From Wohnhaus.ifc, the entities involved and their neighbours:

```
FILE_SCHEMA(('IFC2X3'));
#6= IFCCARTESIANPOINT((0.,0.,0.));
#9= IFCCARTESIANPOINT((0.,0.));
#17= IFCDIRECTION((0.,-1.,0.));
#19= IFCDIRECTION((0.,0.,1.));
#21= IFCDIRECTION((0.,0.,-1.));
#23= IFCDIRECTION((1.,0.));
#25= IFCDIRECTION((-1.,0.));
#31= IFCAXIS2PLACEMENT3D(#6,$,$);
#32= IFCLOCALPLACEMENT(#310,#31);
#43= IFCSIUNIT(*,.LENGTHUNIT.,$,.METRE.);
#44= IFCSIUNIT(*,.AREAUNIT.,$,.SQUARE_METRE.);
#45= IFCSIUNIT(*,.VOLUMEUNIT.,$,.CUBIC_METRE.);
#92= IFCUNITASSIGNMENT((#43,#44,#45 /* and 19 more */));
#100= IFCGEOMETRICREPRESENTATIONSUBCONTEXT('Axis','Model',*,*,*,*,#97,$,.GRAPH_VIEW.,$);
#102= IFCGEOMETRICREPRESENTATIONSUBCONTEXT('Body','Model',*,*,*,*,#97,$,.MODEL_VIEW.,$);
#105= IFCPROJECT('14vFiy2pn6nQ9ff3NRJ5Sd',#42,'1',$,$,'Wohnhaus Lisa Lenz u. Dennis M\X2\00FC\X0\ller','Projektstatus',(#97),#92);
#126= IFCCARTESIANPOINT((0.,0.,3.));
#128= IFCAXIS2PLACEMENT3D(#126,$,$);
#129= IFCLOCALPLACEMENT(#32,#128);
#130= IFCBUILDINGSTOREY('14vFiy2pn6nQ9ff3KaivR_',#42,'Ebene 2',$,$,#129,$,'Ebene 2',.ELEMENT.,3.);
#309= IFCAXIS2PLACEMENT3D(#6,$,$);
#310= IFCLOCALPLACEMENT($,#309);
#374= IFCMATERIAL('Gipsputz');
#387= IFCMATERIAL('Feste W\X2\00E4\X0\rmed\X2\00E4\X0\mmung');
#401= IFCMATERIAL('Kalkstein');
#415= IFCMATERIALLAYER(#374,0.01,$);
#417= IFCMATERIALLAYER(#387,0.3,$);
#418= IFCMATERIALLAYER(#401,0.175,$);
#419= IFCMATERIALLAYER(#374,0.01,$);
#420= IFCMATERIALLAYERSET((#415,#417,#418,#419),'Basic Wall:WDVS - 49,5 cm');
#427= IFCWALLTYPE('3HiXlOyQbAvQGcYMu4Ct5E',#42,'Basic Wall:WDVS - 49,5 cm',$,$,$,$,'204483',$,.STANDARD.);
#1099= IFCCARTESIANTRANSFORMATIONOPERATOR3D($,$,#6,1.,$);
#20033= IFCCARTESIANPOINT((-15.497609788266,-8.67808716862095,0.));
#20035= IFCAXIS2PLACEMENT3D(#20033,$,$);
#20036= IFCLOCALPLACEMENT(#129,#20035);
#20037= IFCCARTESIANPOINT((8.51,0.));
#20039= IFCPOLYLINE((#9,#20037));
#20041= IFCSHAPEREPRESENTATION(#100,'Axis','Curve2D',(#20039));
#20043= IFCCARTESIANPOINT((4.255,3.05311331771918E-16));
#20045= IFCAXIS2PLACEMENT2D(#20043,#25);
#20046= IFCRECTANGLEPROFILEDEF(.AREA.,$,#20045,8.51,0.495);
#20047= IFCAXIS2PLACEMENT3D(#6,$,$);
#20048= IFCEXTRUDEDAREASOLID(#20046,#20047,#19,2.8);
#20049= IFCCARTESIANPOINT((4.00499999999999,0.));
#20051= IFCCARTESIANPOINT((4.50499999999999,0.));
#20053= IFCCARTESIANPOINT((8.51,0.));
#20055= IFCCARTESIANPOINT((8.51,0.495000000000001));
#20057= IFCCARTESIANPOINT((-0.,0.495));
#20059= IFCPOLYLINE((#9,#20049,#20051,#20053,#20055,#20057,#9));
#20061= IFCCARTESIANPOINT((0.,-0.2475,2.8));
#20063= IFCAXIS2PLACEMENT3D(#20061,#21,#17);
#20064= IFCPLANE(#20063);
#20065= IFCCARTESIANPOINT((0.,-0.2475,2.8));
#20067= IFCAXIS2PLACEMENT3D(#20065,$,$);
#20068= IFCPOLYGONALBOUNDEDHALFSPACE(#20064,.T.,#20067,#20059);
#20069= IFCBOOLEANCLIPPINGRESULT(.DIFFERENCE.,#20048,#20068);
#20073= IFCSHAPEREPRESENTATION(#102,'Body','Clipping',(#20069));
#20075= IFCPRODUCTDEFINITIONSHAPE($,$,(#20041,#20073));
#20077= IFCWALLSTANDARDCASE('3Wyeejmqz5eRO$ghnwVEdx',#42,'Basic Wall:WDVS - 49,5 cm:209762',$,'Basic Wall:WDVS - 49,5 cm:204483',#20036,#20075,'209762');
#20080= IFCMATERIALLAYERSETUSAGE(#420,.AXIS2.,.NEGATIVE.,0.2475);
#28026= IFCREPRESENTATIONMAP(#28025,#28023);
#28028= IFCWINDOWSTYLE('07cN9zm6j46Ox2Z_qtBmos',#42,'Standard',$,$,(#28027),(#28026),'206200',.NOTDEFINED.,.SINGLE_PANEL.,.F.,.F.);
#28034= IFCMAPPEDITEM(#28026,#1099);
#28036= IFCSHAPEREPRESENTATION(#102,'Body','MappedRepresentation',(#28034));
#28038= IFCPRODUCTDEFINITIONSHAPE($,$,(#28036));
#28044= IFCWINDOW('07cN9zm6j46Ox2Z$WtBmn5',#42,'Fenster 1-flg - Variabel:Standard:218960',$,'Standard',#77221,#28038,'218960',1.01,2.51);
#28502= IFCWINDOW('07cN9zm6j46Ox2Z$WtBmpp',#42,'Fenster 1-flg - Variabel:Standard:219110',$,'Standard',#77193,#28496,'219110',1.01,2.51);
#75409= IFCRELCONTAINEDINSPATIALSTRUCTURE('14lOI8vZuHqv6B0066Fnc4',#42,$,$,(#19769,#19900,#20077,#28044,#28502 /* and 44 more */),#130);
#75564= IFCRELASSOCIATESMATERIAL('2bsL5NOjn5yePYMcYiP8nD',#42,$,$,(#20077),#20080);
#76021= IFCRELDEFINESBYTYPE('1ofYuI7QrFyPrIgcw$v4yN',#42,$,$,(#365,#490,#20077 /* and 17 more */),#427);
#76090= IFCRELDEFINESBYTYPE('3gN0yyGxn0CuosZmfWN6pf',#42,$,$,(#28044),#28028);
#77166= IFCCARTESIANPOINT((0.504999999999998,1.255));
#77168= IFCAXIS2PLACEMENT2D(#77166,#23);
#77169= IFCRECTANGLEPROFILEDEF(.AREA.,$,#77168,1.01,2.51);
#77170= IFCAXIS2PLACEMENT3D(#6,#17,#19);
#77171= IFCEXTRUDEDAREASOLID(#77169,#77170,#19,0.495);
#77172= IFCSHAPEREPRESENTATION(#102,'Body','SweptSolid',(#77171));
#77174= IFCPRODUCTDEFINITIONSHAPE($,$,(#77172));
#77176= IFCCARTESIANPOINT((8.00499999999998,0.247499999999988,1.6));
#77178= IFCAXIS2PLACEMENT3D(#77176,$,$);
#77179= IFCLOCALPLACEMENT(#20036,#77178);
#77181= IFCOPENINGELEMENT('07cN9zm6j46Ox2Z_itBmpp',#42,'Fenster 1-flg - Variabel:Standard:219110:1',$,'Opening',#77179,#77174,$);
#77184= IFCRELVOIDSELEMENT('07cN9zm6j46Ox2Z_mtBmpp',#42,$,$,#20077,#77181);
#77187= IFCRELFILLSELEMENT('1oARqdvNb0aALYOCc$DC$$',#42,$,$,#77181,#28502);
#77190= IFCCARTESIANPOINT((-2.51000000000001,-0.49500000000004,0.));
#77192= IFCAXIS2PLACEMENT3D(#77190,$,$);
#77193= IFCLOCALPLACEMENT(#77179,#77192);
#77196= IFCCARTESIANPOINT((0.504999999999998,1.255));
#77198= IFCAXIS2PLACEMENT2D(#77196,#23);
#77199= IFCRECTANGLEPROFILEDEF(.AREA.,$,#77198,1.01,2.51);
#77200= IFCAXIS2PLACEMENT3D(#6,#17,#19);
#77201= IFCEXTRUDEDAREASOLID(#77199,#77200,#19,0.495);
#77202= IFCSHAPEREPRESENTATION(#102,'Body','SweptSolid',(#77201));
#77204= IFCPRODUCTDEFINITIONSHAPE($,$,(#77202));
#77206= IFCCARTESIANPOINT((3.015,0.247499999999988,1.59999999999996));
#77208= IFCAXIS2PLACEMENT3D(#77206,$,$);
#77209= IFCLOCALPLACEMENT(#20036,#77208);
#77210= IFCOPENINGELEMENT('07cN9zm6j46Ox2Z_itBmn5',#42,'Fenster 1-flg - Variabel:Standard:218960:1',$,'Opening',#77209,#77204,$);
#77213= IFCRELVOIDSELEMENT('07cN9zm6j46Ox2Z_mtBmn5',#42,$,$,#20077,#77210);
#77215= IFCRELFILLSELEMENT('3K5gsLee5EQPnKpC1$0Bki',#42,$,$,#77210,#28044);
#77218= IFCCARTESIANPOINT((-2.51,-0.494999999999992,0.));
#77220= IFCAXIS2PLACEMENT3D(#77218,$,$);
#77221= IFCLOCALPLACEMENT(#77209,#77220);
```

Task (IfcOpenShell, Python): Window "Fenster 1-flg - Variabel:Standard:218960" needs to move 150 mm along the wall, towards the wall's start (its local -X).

```python
import ifcopenshell
import ifcopenshell.api.geometry
import ifcopenshell.util.placement

model = ifcopenshell.open("Wohnhaus.ifc")

window = model.by_id(28044)
opening = window.FillsVoids[0].RelatingOpeningElement
wall = opening.VoidsElements[0].RelatingBuildingElement

wall_matrix = ifcopenshell.util.placement.get_local_placement(wall.ObjectPlacement)
shift = wall_matrix[:3, 0] * -0.15
before = ifcopenshell.util.placement.get_local_placement(window.ObjectPlacement)[:3, 3].copy()

# The window is placed relative to its opening, so it follows when the opening moves.
matrix = ifcopenshell.util.placement.get_local_placement(opening.ObjectPlacement)
matrix[:3, 3] += shift
ifcopenshell.api.geometry.edit_object_placement(
    model, product=opening, matrix=matrix, is_si=False, should_transform_children=True
)

after = ifcopenshell.util.placement.get_local_placement(window.ObjectPlacement)[:3, 3]
print("window moved by", (after - before).round(3) + 0.0)

model.write("Wohnhaus-out.ifc")
```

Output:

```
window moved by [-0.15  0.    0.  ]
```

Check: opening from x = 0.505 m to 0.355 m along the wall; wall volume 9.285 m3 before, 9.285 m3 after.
